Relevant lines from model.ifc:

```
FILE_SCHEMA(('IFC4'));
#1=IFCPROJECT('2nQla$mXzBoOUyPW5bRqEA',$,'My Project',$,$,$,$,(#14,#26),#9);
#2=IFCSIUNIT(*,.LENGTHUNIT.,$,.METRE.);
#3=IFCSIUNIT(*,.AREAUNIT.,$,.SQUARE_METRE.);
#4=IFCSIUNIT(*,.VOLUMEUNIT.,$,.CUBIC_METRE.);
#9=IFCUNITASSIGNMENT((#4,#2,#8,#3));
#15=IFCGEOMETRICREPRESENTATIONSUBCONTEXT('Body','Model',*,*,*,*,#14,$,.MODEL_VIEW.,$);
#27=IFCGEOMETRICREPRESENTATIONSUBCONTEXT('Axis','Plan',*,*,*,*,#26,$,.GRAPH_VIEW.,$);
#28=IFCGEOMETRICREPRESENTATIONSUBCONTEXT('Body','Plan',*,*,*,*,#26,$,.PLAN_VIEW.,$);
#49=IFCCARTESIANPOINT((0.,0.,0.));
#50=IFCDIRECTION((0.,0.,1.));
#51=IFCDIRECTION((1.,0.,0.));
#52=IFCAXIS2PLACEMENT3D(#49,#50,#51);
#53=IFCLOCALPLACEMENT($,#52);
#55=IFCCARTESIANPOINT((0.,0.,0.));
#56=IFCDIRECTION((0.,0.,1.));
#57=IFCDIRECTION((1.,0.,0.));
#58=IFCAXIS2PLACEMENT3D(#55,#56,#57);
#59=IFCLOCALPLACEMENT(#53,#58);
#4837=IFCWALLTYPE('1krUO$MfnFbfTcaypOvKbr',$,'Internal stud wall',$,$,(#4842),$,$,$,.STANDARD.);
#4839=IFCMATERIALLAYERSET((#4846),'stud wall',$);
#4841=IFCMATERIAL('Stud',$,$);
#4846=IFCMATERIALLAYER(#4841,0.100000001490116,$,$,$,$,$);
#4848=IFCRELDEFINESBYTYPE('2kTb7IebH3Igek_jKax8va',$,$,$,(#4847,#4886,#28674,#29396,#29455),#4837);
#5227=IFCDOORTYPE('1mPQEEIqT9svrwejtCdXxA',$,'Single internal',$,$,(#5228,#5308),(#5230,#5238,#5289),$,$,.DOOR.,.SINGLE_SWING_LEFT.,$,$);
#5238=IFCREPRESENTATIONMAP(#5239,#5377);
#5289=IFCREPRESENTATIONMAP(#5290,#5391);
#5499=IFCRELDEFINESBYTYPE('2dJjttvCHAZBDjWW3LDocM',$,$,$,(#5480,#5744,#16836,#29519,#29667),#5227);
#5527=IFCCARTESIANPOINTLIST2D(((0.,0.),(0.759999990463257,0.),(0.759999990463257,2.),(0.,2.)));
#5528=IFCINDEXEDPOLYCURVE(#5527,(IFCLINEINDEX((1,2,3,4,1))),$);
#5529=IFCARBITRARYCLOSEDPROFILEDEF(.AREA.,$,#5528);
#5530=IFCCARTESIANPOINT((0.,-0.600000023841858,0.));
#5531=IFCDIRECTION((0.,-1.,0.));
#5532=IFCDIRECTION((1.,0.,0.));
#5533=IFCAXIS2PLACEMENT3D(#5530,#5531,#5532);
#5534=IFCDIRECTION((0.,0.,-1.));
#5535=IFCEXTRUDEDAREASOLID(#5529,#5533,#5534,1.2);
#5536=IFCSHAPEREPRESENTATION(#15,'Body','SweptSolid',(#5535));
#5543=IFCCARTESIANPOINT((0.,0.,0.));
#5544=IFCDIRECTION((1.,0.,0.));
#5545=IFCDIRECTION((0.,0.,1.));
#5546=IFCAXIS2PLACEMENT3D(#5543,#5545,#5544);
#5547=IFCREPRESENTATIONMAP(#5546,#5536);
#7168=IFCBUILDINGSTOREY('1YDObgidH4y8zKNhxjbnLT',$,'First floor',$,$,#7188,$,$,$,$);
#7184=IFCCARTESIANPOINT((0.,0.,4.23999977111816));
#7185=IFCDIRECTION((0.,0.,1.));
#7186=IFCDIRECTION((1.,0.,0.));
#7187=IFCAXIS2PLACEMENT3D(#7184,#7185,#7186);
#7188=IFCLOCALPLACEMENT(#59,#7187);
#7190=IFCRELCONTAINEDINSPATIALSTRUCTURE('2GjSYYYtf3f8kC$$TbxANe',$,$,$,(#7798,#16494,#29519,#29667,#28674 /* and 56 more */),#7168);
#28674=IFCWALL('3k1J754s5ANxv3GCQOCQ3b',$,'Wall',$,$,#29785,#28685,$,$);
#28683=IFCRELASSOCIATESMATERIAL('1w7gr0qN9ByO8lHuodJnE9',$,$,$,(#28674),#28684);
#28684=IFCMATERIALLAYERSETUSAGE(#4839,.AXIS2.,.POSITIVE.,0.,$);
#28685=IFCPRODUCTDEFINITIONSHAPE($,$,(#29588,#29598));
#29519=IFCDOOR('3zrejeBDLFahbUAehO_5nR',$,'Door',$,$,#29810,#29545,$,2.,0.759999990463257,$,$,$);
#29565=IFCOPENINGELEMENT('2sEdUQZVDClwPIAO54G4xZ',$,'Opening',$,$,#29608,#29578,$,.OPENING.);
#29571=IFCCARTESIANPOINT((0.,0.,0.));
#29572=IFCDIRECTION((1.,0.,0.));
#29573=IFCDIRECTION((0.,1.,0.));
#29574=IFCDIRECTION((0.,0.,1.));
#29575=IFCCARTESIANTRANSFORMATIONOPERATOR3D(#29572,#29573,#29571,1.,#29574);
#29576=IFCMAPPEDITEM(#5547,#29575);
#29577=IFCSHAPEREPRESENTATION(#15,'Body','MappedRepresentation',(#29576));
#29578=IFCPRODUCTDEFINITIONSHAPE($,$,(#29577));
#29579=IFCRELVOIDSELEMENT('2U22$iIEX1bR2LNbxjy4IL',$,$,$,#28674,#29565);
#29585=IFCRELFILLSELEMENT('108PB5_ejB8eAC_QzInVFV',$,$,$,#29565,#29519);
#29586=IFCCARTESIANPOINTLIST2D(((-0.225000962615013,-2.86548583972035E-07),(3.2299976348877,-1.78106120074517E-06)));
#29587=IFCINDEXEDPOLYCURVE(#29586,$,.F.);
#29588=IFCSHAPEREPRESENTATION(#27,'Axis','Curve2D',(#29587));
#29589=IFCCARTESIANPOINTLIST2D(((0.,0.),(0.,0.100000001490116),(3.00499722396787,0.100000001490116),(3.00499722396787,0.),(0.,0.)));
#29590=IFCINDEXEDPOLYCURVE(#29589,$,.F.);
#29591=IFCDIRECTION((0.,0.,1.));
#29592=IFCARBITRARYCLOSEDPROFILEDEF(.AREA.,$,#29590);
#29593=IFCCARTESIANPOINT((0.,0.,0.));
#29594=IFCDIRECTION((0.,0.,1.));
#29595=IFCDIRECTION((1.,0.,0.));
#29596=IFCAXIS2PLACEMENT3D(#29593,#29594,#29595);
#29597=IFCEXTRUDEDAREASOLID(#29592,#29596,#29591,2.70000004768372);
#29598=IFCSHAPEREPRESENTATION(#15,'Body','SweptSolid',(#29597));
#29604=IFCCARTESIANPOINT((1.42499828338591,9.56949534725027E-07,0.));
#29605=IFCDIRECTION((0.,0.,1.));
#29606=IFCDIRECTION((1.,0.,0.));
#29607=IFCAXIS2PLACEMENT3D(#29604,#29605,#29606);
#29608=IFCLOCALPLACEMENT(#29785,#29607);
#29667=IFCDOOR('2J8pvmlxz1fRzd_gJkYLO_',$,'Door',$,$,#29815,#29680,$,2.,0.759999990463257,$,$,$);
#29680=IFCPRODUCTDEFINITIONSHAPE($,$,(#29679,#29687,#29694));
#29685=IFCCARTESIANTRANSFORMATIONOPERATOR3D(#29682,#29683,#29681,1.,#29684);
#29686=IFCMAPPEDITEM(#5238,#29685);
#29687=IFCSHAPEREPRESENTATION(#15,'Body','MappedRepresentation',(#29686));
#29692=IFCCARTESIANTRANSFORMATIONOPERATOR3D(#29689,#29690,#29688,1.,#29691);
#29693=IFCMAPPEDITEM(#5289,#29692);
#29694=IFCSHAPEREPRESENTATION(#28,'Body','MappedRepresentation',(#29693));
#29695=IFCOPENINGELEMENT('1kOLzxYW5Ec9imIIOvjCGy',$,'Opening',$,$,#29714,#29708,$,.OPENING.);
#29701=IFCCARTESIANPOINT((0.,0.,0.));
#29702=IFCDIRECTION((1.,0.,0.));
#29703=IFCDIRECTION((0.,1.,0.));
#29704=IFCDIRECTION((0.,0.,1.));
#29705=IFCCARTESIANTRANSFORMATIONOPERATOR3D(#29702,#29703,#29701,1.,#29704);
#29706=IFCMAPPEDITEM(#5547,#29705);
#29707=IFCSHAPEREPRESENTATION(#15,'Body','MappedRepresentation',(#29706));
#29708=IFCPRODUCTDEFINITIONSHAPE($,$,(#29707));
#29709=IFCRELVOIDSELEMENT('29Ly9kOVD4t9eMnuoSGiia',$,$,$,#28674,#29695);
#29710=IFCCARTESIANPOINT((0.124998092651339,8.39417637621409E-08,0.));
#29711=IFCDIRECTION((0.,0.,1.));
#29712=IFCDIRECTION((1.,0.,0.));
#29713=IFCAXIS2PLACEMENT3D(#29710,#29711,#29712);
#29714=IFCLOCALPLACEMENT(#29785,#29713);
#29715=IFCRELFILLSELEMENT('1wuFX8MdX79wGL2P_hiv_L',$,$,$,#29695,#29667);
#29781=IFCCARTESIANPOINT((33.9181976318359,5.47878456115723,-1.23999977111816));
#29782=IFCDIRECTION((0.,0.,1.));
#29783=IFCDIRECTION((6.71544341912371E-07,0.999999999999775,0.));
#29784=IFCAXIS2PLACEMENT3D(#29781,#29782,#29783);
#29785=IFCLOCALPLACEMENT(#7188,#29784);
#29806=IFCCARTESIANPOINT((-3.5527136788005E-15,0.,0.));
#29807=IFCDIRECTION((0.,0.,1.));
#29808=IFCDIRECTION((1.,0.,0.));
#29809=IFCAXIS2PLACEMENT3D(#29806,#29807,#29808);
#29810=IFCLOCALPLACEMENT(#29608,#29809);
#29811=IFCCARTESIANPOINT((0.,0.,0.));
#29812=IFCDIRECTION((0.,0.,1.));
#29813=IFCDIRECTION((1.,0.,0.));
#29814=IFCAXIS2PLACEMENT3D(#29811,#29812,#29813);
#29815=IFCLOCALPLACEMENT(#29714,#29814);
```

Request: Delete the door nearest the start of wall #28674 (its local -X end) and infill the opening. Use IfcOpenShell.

```python
import ifcopenshell
import ifcopenshell.api.feature
import ifcopenshell.api.root
import ifcopenshell.geom
import ifcopenshell.util.shape

model = ifcopenshell.open("model.ifc")
settings = ifcopenshell.geom.settings()


def volume(element):
    """Net volume in cubic metres, openings subtracted."""
    shape = ifcopenshell.geom.create_shape(settings, element)
    return ifcopenshell.util.shape.get_volume(shape.geometry)


door = model.by_id(29667)
opening = door.FillsVoids[0].RelatingOpeningElement
wall = opening.VoidsElements[0].RelatingBuildingElement
before = volume(wall)

ifcopenshell.api.root.remove_product(model, product=door)
ifcopenshell.api.feature.remove_feature(model, feature=opening)

after = volume(wall)

print(f"wall volume {before:.3f} -> {after:.3f} m3")

model.write("model_edited.ifc")
```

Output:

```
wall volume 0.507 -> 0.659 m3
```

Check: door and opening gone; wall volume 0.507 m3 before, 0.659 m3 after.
